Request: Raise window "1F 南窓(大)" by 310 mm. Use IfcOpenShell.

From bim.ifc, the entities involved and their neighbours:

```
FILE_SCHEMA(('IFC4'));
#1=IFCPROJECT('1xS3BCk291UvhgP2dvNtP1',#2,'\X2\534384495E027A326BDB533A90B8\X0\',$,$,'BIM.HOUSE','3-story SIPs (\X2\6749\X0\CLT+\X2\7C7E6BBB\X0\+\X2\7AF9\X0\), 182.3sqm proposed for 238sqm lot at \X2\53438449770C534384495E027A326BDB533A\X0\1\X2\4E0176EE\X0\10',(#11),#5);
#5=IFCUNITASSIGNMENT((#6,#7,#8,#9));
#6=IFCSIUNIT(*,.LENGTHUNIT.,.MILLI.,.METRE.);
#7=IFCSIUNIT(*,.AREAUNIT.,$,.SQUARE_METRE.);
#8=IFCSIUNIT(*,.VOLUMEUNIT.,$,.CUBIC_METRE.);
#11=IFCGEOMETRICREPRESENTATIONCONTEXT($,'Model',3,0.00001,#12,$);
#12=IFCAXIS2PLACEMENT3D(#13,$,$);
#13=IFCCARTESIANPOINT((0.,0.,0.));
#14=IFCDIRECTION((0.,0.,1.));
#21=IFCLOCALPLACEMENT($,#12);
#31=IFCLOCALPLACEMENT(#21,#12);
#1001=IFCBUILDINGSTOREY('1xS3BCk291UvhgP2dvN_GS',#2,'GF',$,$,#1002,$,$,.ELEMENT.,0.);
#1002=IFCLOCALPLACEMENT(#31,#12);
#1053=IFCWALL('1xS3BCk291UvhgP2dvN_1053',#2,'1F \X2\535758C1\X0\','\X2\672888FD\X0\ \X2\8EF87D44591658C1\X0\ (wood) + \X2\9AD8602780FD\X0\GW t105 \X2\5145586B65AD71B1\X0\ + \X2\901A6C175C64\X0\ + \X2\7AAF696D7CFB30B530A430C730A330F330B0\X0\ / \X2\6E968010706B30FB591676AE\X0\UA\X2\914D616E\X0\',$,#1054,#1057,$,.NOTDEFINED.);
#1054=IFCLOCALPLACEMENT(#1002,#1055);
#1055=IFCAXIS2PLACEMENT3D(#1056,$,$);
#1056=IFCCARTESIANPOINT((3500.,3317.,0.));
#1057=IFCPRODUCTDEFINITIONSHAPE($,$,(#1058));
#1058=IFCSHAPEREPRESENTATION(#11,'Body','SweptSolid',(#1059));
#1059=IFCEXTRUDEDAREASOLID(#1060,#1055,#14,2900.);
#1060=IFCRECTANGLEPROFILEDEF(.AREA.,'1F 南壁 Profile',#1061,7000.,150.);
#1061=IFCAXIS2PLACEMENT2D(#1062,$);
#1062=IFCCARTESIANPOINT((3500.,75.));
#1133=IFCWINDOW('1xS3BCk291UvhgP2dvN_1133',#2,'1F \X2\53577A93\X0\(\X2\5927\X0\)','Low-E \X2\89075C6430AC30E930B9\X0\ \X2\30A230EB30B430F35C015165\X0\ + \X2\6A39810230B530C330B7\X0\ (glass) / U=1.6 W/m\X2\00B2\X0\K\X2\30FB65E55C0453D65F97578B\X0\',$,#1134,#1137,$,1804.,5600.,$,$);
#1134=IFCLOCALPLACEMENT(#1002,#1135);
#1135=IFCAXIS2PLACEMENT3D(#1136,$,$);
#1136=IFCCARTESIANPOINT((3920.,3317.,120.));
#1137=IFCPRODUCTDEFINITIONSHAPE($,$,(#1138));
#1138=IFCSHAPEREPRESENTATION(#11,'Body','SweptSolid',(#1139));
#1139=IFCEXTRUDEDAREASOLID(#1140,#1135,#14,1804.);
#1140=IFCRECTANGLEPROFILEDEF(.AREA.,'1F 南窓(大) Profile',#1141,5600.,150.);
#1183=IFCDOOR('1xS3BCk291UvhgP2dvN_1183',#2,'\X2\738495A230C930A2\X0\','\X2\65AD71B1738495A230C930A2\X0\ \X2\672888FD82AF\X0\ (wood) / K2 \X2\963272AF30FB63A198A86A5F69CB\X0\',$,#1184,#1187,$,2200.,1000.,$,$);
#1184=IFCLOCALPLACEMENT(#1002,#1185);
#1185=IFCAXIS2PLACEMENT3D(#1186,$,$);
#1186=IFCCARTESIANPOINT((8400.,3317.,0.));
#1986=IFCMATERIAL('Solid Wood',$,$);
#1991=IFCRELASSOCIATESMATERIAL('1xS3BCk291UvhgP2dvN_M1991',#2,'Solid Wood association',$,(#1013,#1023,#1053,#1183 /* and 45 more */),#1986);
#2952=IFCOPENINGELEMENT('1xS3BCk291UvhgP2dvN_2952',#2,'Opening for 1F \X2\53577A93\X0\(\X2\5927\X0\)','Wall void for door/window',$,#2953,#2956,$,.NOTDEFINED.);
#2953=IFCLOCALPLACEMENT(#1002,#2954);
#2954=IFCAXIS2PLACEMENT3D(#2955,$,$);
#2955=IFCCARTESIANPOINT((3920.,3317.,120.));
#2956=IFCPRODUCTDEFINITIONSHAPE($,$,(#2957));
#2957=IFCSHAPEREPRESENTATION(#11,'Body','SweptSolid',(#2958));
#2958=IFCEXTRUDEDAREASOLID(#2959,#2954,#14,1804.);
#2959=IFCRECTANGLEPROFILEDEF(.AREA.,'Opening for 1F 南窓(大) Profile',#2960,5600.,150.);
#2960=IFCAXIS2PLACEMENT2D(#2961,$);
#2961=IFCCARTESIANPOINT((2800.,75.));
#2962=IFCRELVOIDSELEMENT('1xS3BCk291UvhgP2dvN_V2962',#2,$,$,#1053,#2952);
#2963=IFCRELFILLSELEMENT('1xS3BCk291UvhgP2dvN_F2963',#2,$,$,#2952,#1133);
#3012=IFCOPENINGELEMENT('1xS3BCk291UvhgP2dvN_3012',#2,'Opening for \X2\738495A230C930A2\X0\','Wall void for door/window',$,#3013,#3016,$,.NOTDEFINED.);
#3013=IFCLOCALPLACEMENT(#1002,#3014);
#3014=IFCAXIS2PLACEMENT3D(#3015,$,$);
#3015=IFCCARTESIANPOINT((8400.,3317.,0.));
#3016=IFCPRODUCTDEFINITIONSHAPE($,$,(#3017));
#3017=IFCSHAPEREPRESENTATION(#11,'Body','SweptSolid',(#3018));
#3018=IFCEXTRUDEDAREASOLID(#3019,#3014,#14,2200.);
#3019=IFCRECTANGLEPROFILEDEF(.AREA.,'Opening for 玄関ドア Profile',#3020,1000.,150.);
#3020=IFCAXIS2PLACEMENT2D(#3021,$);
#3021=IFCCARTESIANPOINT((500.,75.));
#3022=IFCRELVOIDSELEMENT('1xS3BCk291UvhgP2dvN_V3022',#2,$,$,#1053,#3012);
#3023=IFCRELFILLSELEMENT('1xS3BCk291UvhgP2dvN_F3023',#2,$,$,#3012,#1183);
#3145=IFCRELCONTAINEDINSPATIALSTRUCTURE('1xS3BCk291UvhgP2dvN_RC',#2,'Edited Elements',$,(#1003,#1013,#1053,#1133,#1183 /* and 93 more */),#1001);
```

```python
import numpy as np
import ifcopenshell
import ifcopenshell.api.geometry
import ifcopenshell.util.placement
import ifcopenshell.util.unit

model = ifcopenshell.open("bim.ifc")
unit_scale = ifcopenshell.util.unit.calculate_unit_scale(model)

window = model.by_id(1133)
opening = window.FillsVoids[0].RelatingOpeningElement
dz = 0.31 / unit_scale

shift = np.array([0.0, 0.0, dz])
# The window is not placed relative to its opening, so move both.
for product in (opening, window):
    matrix = ifcopenshell.util.placement.get_local_placement(product.ObjectPlacement)
    matrix[:3, 3] += shift
    ifcopenshell.api.geometry.edit_object_placement(model, product=product, matrix=matrix, is_si=False)

print(f"moved by {dz * unit_scale:+.3f} m")

model.write("bim_v2.ifc")
```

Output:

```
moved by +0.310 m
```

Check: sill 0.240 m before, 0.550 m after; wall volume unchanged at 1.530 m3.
